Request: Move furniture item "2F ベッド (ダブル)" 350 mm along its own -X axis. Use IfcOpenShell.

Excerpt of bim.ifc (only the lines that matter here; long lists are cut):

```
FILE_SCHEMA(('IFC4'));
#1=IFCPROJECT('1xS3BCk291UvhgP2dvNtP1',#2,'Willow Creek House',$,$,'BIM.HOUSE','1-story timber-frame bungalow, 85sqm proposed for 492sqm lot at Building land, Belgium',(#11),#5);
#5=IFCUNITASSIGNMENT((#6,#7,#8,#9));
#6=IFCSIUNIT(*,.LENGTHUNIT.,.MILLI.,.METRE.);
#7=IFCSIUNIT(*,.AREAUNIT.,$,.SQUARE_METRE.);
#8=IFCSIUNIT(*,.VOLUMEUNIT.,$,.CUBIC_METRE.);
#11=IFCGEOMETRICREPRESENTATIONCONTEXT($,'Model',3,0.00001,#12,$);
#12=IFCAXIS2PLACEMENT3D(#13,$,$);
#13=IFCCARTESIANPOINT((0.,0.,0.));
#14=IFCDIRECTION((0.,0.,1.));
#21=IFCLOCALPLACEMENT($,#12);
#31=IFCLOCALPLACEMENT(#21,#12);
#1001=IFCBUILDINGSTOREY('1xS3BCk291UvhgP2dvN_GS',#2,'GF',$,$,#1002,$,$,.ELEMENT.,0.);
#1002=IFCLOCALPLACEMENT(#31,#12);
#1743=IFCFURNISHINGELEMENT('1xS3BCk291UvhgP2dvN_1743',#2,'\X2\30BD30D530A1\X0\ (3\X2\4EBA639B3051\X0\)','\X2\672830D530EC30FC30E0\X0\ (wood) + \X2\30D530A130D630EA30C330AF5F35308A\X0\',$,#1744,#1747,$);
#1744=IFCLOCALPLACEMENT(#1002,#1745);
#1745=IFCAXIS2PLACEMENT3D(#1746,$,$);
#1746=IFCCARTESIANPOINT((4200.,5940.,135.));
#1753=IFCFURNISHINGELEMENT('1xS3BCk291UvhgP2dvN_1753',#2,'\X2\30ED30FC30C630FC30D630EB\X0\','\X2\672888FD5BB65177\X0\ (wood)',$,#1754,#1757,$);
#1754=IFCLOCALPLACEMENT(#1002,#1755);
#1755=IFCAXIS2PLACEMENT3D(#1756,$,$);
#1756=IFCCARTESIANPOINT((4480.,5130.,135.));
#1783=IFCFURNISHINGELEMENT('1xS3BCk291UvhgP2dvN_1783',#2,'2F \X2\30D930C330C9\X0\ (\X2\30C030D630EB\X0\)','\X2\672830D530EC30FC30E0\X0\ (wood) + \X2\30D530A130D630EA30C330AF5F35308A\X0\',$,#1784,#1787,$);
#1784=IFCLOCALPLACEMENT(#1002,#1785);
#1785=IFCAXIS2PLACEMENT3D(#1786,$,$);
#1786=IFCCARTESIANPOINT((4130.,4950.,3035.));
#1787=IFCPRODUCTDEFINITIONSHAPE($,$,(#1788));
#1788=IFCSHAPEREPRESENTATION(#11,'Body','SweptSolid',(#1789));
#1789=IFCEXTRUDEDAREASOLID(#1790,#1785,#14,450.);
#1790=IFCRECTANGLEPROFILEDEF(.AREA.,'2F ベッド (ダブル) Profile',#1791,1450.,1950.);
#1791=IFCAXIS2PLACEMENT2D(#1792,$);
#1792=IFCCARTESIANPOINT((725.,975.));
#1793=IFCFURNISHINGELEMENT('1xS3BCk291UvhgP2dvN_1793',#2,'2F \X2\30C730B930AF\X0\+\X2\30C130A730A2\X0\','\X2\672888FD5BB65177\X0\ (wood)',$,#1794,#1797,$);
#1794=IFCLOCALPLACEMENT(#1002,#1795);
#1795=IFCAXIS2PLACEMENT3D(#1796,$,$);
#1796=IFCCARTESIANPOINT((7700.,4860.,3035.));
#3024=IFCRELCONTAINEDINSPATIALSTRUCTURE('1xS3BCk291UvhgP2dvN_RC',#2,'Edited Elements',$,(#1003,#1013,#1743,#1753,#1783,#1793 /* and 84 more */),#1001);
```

```python
import ifcopenshell
import ifcopenshell.api.geometry
import ifcopenshell.util.placement
import ifcopenshell.util.unit

model = ifcopenshell.open("bim.ifc")
unit_scale = ifcopenshell.util.unit.calculate_unit_scale(model)

item = model.by_id(1783)
matrix = ifcopenshell.util.placement.get_local_placement(item.ObjectPlacement)
matrix[:3, 3] -= matrix[:3, 0] * 0.35 / unit_scale
ifcopenshell.api.geometry.edit_object_placement(model, product=item, matrix=matrix, is_si=False)

print(ifcopenshell.util.placement.get_local_placement(item.ObjectPlacement).round(3) + 0.0)

model.write("bim_v2.ifc")
```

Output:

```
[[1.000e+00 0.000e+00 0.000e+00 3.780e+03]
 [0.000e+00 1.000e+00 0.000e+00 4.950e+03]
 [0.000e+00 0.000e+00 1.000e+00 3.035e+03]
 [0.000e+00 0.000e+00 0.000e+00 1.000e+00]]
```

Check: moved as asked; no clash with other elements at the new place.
